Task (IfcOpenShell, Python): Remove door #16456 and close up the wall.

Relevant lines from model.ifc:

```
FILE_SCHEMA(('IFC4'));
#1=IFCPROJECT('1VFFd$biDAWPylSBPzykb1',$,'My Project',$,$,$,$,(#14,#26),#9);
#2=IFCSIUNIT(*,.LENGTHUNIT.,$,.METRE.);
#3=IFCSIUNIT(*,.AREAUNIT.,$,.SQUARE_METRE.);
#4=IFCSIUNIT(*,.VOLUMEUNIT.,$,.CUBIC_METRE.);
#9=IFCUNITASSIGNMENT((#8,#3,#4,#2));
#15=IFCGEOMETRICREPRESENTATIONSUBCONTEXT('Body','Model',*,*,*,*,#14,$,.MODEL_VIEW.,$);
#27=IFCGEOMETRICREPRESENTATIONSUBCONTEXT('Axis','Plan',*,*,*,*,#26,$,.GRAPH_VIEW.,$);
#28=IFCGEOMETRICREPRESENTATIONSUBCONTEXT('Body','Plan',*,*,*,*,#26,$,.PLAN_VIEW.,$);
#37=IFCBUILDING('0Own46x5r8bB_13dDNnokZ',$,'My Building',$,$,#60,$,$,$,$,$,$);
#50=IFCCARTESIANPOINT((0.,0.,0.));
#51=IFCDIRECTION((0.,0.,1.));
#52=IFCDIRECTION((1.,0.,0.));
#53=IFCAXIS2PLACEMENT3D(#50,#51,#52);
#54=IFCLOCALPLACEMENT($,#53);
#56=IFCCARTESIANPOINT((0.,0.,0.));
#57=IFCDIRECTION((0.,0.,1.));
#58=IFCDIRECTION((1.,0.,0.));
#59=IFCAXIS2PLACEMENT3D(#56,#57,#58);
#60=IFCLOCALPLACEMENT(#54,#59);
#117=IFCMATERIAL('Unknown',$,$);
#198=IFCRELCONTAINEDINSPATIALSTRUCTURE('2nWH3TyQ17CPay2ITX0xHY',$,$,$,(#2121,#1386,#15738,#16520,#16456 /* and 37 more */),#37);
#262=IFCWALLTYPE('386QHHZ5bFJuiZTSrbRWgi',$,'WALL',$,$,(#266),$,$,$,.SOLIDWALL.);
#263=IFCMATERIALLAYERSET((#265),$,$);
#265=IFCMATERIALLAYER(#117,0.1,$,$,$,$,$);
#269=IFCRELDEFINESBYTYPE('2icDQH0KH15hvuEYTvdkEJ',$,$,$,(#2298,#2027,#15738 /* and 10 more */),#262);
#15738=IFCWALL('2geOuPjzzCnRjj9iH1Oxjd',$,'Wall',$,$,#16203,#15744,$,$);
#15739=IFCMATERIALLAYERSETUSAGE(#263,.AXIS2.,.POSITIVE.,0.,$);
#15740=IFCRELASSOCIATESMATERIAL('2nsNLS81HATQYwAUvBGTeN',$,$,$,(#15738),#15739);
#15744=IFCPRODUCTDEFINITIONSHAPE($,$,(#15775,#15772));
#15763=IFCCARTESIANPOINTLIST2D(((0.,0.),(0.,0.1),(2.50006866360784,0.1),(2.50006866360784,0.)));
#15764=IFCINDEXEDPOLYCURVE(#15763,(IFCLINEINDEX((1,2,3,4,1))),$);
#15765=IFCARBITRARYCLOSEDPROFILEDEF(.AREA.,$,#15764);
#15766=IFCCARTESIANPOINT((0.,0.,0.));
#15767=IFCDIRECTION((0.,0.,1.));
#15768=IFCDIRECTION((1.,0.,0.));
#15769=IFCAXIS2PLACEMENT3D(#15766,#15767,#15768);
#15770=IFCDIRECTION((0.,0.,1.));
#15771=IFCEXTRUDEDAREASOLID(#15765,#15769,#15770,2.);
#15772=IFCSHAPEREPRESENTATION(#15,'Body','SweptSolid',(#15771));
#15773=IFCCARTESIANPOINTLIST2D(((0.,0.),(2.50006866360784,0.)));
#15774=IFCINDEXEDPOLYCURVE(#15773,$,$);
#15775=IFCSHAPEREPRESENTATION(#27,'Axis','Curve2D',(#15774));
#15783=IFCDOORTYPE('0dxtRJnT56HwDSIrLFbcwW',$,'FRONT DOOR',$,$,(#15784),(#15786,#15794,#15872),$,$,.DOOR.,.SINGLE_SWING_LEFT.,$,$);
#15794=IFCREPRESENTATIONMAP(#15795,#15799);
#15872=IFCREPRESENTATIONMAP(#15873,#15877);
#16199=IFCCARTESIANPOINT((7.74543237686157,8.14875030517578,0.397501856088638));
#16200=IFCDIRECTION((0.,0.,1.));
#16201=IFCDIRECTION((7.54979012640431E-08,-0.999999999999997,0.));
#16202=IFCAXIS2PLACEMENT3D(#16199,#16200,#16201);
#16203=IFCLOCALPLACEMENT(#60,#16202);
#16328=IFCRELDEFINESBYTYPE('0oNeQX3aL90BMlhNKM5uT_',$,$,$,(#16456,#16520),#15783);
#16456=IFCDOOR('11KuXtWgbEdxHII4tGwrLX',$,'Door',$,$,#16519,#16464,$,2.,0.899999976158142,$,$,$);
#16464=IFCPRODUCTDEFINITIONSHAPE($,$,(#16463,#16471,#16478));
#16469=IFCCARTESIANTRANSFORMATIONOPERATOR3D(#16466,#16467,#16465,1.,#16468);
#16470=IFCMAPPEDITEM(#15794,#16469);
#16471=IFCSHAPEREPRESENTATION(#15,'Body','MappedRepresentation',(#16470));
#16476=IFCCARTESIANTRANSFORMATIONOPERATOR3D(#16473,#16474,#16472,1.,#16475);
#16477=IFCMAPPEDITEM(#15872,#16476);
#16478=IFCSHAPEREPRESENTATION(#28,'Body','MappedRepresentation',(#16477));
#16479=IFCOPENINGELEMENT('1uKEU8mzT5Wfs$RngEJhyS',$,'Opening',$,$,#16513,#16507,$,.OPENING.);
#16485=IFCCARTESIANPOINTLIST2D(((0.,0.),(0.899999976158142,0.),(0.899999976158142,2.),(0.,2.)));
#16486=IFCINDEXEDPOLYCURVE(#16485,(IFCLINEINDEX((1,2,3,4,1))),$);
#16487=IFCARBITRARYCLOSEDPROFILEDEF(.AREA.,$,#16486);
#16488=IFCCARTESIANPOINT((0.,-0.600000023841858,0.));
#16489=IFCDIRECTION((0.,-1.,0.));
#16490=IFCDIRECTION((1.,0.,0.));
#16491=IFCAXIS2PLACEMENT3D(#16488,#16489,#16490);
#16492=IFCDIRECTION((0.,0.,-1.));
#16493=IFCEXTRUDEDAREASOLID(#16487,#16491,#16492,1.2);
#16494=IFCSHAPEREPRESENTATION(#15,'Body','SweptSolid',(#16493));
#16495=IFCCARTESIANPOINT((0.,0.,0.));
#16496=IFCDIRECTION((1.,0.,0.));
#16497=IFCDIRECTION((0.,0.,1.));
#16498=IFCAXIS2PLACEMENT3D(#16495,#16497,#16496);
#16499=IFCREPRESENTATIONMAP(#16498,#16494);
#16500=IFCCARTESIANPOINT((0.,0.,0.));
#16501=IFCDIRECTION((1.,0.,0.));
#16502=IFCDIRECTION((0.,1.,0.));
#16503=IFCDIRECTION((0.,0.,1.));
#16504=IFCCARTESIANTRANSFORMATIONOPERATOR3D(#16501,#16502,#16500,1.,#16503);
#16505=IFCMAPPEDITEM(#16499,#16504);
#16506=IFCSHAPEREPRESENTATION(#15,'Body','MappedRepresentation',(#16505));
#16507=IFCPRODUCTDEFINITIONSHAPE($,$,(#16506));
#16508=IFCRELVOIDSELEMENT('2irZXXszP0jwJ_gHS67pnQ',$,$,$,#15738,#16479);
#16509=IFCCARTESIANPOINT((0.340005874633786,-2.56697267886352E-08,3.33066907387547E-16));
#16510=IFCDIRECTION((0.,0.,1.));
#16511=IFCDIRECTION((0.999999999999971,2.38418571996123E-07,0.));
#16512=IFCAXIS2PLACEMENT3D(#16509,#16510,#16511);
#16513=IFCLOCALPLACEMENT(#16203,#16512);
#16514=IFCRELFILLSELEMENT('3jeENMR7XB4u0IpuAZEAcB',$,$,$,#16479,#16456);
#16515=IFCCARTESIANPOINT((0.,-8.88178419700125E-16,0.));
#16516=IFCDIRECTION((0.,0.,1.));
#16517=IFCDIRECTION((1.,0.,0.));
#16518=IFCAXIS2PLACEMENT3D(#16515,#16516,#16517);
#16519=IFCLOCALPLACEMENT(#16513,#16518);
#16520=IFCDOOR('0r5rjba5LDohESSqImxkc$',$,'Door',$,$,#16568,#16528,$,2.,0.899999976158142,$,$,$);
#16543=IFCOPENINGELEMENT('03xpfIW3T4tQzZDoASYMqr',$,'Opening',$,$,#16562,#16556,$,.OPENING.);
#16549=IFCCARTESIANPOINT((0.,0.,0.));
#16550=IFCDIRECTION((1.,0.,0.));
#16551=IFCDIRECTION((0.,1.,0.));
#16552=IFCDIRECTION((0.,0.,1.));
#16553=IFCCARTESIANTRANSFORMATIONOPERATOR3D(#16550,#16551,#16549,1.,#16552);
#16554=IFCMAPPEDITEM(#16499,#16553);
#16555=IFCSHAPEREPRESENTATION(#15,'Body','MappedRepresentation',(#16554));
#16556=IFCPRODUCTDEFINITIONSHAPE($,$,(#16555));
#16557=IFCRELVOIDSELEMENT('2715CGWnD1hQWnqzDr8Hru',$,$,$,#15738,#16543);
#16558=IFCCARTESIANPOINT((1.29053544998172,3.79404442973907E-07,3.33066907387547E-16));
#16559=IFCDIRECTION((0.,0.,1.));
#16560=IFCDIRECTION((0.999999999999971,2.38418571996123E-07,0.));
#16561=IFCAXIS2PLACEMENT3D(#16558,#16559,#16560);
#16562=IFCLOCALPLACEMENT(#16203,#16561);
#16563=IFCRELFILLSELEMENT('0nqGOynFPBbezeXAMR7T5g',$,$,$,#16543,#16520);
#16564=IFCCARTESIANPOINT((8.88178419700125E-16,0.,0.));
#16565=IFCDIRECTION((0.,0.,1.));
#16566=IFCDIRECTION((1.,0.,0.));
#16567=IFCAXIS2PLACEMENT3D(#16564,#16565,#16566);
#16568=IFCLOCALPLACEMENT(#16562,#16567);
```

```python
import ifcopenshell
import ifcopenshell.api.feature
import ifcopenshell.api.root
import ifcopenshell.geom
import ifcopenshell.util.shape

model = ifcopenshell.open("model.ifc")
settings = ifcopenshell.geom.settings()


def volume(element):
    """Net volume in cubic metres, openings subtracted."""
    shape = ifcopenshell.geom.create_shape(settings, element)
    return ifcopenshell.util.shape.get_volume(shape.geometry)


door = model.by_guid("11KuXtWgbEdxHII4tGwrLX")
opening = door.FillsVoids[0].RelatingOpeningElement
wall = opening.VoidsElements[0].RelatingBuildingElement
before = volume(wall)

ifcopenshell.api.root.remove_product(model, product=door)
ifcopenshell.api.feature.remove_feature(model, feature=opening)

after = volume(wall)

print(f"wall volume {before:.3f} -> {after:.3f} m3")

model.write("model_edited.ifc")
```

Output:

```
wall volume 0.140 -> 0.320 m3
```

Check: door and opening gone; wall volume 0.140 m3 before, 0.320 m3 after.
